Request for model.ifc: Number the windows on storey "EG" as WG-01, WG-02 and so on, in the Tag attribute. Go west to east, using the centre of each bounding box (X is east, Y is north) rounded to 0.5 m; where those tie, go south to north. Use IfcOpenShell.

First a look at what the model holds.

```python
import ifcopenshell
import ifcopenshell.util.element
import ifcopenshell.util.placement

model = ifcopenshell.open("model.ifc")
print(model.schema)
storey = next(s for s in model.by_type("IfcBuildingStorey") if s.Name == "EG")
windows = [e for e in ifcopenshell.util.element.get_decomposition(storey) if e.is_a("IfcWindow")]
for e in sorted(windows, key=lambda e: e.id()):
    origin = ifcopenshell.util.placement.get_local_placement(e.ObjectPlacement)[:3, 3]
    print(e.id(), e.Tag, e.Name, origin.round(2) + 0.0, sep=" | ")
```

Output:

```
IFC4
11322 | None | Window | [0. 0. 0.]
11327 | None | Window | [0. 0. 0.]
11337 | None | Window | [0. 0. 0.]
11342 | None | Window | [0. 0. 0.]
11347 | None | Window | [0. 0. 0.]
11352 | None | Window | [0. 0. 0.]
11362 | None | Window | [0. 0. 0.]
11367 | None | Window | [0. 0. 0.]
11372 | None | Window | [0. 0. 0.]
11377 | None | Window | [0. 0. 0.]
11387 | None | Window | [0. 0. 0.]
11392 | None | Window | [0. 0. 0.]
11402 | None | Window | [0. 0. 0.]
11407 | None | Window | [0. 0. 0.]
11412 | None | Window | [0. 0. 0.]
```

```python
import ifcopenshell
import ifcopenshell.geom
import ifcopenshell.util.element
import ifcopenshell.util.shape

model = ifcopenshell.open("model.ifc")
settings = ifcopenshell.geom.settings()
settings.set("use-world-coords", True)


def centre(element):
    shape = ifcopenshell.geom.create_shape(settings, element)
    return ifcopenshell.util.shape.get_bbox_centroid(shape.geometry)


storey = next(s for s in model.by_type("IfcBuildingStorey") if s.Name == "EG")
windows = [e for e in ifcopenshell.util.element.get_decomposition(storey) if e.is_a("IfcWindow")]

# Insertion points can sit at a corner or the storey origin, so sort by the geometry (in metres).
centres = {e: centre(e) for e in windows}
windows.sort(key=lambda e: (round(centres[e][0] / 0.5), centres[e][1]))

for i, e in enumerate(windows, start=1):
    number = f"WG-{i:02d}"
    e.Tag = number
    print(e.id(), number)

model.write("model_updated.ifc")
```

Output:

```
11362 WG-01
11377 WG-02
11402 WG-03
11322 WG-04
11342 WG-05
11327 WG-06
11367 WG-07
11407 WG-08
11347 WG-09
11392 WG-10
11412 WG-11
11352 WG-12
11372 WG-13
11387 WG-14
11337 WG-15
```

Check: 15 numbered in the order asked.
